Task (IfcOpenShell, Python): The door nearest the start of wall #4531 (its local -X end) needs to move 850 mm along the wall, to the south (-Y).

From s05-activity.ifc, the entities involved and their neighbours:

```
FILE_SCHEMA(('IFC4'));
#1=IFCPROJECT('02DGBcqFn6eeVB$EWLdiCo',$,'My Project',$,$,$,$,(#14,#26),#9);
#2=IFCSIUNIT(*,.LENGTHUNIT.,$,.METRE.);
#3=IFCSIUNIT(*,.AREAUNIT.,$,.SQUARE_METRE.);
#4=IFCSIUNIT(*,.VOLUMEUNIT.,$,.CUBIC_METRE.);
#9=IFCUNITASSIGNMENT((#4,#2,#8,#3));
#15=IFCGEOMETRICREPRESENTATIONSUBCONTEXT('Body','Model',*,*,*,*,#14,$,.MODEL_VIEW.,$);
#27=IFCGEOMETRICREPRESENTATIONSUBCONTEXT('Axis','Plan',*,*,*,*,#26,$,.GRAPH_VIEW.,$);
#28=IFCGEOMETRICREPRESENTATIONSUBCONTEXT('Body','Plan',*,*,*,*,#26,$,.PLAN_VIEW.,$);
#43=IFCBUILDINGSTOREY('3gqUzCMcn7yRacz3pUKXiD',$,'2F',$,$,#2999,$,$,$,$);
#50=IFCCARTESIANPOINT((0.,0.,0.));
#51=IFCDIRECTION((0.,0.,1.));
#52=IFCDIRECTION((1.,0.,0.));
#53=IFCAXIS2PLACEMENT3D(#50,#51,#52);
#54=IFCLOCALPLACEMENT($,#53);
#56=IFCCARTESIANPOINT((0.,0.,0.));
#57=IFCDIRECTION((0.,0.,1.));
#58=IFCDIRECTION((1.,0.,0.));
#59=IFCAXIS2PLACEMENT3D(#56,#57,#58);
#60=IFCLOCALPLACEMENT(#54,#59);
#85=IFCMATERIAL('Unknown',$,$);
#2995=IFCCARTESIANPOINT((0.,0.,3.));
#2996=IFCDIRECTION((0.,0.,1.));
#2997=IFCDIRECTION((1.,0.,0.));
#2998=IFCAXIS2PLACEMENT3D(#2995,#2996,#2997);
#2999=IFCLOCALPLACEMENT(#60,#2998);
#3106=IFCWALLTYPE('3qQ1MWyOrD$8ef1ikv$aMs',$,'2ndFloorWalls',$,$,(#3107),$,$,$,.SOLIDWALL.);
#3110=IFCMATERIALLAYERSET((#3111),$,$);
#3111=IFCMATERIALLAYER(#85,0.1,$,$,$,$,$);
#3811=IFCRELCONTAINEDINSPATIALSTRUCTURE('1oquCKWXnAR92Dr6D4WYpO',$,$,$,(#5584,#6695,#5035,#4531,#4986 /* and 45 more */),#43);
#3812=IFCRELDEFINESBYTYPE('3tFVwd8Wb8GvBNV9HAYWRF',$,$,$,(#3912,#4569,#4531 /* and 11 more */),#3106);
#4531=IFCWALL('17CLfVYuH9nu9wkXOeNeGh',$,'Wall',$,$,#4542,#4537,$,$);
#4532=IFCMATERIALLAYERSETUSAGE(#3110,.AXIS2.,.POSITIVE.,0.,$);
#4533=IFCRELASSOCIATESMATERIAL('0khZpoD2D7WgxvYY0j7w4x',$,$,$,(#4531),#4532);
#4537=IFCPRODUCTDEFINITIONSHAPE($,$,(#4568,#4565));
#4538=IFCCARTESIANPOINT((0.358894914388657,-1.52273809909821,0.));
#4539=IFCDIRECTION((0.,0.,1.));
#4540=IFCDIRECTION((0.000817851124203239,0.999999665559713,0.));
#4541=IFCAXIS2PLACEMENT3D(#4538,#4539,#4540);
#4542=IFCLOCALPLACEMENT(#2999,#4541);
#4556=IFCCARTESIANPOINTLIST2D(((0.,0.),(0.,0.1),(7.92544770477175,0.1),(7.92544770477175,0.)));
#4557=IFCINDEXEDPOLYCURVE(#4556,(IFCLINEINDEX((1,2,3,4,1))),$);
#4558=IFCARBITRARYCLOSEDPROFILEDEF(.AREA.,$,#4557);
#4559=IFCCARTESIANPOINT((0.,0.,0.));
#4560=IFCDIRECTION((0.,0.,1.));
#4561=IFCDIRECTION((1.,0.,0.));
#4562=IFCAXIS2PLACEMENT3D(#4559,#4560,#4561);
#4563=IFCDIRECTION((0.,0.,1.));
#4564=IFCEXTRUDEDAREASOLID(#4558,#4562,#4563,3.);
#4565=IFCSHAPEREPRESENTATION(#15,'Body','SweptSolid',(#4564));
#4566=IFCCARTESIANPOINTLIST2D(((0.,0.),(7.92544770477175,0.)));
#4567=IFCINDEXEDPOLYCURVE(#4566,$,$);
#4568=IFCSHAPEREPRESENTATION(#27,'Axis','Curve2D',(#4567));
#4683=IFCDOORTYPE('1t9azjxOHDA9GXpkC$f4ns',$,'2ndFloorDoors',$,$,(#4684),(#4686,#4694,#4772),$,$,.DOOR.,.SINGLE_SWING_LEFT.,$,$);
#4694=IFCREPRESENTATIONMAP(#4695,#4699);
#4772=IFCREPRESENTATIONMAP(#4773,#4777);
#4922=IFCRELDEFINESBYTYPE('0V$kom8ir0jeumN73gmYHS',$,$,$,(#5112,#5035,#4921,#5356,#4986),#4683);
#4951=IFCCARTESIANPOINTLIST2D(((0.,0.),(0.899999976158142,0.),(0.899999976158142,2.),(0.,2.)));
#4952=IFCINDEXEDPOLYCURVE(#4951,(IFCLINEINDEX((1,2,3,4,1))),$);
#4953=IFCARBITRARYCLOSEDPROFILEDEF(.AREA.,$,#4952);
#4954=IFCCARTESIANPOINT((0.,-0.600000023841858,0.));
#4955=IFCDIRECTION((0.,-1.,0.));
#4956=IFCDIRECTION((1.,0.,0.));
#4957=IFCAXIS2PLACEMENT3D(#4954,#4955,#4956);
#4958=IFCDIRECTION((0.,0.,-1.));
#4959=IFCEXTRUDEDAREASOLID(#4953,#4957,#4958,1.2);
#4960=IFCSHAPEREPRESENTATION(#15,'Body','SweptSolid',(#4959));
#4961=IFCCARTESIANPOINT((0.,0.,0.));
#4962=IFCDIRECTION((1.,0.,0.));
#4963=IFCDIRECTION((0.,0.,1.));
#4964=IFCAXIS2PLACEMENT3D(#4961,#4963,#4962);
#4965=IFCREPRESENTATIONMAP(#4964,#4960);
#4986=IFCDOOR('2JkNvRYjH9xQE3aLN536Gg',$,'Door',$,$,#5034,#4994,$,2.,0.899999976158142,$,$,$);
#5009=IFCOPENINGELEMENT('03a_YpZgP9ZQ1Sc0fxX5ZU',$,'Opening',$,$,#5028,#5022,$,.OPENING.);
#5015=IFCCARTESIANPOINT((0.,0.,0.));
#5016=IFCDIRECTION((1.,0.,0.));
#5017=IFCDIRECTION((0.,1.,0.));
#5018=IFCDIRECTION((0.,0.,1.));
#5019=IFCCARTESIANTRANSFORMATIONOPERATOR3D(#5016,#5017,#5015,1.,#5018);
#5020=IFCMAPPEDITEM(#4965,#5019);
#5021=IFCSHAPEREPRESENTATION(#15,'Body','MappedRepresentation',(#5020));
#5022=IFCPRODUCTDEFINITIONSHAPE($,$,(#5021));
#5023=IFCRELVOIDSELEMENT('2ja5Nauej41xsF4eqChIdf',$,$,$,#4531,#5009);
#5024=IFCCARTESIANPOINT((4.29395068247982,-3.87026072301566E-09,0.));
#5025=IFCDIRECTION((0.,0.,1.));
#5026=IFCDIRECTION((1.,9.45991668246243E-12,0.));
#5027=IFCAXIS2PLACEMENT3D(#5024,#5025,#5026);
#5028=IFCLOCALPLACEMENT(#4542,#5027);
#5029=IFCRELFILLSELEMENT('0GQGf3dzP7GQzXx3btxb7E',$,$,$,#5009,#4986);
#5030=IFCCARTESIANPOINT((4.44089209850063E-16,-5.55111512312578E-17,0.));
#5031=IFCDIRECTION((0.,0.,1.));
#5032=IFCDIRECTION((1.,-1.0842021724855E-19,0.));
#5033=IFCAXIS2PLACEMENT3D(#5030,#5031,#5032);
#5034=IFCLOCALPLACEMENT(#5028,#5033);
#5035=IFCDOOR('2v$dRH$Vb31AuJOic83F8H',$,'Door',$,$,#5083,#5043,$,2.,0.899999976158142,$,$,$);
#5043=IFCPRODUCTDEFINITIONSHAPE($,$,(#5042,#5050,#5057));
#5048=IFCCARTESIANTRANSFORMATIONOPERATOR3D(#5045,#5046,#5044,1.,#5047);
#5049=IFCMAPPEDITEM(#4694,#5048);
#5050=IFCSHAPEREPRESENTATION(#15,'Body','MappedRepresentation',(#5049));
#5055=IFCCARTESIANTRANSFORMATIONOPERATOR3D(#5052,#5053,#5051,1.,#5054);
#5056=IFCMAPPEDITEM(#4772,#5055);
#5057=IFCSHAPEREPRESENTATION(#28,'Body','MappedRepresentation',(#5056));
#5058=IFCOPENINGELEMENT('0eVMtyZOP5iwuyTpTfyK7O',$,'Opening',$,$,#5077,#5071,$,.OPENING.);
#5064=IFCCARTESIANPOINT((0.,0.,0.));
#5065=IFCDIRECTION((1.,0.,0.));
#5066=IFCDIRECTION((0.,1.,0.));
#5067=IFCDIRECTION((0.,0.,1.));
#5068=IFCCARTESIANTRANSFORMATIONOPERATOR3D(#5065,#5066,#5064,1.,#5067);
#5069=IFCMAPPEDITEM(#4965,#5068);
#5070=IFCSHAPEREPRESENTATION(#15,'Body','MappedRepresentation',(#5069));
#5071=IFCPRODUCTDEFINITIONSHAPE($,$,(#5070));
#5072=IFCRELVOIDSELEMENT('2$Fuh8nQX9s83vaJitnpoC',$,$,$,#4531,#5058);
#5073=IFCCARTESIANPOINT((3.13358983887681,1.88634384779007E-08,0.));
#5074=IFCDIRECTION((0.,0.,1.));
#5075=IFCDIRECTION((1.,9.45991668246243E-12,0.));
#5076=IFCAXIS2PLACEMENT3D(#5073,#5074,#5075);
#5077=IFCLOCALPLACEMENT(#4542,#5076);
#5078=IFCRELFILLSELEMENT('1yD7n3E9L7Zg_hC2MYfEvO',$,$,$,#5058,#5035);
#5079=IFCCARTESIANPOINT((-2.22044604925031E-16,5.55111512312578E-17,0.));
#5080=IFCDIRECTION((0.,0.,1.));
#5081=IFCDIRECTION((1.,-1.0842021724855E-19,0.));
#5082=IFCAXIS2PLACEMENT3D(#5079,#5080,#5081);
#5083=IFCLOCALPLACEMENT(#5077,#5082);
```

```python
import ifcopenshell
import ifcopenshell.api.geometry
import ifcopenshell.util.placement
import ifcopenshell.util.unit

model = ifcopenshell.open("s05-activity.ifc")
unit_scale = ifcopenshell.util.unit.calculate_unit_scale(model)

door = model.by_guid("2v$dRH$Vb31AuJOic83F8H")
opening = door.FillsVoids[0].RelatingOpeningElement
wall = opening.VoidsElements[0].RelatingBuildingElement

wall_matrix = ifcopenshell.util.placement.get_local_placement(wall.ObjectPlacement)
shift = wall_matrix[:3, 0] * -0.85 / unit_scale
before = ifcopenshell.util.placement.get_local_placement(door.ObjectPlacement)[:3, 3].copy()

# The door is placed relative to its opening, so it follows when the opening moves.
matrix = ifcopenshell.util.placement.get_local_placement(opening.ObjectPlacement)
matrix[:3, 3] += shift
ifcopenshell.api.geometry.edit_object_placement(
    model, product=opening, matrix=matrix, is_si=False, should_transform_children=True
)

after = ifcopenshell.util.placement.get_local_placement(door.ObjectPlacement)[:3, 3]
print("door moved by", (after - before).round(3) + 0.0)

model.write("s05-activity_rev.ifc")
```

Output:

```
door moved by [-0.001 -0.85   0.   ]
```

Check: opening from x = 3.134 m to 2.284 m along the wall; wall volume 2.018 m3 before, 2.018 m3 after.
